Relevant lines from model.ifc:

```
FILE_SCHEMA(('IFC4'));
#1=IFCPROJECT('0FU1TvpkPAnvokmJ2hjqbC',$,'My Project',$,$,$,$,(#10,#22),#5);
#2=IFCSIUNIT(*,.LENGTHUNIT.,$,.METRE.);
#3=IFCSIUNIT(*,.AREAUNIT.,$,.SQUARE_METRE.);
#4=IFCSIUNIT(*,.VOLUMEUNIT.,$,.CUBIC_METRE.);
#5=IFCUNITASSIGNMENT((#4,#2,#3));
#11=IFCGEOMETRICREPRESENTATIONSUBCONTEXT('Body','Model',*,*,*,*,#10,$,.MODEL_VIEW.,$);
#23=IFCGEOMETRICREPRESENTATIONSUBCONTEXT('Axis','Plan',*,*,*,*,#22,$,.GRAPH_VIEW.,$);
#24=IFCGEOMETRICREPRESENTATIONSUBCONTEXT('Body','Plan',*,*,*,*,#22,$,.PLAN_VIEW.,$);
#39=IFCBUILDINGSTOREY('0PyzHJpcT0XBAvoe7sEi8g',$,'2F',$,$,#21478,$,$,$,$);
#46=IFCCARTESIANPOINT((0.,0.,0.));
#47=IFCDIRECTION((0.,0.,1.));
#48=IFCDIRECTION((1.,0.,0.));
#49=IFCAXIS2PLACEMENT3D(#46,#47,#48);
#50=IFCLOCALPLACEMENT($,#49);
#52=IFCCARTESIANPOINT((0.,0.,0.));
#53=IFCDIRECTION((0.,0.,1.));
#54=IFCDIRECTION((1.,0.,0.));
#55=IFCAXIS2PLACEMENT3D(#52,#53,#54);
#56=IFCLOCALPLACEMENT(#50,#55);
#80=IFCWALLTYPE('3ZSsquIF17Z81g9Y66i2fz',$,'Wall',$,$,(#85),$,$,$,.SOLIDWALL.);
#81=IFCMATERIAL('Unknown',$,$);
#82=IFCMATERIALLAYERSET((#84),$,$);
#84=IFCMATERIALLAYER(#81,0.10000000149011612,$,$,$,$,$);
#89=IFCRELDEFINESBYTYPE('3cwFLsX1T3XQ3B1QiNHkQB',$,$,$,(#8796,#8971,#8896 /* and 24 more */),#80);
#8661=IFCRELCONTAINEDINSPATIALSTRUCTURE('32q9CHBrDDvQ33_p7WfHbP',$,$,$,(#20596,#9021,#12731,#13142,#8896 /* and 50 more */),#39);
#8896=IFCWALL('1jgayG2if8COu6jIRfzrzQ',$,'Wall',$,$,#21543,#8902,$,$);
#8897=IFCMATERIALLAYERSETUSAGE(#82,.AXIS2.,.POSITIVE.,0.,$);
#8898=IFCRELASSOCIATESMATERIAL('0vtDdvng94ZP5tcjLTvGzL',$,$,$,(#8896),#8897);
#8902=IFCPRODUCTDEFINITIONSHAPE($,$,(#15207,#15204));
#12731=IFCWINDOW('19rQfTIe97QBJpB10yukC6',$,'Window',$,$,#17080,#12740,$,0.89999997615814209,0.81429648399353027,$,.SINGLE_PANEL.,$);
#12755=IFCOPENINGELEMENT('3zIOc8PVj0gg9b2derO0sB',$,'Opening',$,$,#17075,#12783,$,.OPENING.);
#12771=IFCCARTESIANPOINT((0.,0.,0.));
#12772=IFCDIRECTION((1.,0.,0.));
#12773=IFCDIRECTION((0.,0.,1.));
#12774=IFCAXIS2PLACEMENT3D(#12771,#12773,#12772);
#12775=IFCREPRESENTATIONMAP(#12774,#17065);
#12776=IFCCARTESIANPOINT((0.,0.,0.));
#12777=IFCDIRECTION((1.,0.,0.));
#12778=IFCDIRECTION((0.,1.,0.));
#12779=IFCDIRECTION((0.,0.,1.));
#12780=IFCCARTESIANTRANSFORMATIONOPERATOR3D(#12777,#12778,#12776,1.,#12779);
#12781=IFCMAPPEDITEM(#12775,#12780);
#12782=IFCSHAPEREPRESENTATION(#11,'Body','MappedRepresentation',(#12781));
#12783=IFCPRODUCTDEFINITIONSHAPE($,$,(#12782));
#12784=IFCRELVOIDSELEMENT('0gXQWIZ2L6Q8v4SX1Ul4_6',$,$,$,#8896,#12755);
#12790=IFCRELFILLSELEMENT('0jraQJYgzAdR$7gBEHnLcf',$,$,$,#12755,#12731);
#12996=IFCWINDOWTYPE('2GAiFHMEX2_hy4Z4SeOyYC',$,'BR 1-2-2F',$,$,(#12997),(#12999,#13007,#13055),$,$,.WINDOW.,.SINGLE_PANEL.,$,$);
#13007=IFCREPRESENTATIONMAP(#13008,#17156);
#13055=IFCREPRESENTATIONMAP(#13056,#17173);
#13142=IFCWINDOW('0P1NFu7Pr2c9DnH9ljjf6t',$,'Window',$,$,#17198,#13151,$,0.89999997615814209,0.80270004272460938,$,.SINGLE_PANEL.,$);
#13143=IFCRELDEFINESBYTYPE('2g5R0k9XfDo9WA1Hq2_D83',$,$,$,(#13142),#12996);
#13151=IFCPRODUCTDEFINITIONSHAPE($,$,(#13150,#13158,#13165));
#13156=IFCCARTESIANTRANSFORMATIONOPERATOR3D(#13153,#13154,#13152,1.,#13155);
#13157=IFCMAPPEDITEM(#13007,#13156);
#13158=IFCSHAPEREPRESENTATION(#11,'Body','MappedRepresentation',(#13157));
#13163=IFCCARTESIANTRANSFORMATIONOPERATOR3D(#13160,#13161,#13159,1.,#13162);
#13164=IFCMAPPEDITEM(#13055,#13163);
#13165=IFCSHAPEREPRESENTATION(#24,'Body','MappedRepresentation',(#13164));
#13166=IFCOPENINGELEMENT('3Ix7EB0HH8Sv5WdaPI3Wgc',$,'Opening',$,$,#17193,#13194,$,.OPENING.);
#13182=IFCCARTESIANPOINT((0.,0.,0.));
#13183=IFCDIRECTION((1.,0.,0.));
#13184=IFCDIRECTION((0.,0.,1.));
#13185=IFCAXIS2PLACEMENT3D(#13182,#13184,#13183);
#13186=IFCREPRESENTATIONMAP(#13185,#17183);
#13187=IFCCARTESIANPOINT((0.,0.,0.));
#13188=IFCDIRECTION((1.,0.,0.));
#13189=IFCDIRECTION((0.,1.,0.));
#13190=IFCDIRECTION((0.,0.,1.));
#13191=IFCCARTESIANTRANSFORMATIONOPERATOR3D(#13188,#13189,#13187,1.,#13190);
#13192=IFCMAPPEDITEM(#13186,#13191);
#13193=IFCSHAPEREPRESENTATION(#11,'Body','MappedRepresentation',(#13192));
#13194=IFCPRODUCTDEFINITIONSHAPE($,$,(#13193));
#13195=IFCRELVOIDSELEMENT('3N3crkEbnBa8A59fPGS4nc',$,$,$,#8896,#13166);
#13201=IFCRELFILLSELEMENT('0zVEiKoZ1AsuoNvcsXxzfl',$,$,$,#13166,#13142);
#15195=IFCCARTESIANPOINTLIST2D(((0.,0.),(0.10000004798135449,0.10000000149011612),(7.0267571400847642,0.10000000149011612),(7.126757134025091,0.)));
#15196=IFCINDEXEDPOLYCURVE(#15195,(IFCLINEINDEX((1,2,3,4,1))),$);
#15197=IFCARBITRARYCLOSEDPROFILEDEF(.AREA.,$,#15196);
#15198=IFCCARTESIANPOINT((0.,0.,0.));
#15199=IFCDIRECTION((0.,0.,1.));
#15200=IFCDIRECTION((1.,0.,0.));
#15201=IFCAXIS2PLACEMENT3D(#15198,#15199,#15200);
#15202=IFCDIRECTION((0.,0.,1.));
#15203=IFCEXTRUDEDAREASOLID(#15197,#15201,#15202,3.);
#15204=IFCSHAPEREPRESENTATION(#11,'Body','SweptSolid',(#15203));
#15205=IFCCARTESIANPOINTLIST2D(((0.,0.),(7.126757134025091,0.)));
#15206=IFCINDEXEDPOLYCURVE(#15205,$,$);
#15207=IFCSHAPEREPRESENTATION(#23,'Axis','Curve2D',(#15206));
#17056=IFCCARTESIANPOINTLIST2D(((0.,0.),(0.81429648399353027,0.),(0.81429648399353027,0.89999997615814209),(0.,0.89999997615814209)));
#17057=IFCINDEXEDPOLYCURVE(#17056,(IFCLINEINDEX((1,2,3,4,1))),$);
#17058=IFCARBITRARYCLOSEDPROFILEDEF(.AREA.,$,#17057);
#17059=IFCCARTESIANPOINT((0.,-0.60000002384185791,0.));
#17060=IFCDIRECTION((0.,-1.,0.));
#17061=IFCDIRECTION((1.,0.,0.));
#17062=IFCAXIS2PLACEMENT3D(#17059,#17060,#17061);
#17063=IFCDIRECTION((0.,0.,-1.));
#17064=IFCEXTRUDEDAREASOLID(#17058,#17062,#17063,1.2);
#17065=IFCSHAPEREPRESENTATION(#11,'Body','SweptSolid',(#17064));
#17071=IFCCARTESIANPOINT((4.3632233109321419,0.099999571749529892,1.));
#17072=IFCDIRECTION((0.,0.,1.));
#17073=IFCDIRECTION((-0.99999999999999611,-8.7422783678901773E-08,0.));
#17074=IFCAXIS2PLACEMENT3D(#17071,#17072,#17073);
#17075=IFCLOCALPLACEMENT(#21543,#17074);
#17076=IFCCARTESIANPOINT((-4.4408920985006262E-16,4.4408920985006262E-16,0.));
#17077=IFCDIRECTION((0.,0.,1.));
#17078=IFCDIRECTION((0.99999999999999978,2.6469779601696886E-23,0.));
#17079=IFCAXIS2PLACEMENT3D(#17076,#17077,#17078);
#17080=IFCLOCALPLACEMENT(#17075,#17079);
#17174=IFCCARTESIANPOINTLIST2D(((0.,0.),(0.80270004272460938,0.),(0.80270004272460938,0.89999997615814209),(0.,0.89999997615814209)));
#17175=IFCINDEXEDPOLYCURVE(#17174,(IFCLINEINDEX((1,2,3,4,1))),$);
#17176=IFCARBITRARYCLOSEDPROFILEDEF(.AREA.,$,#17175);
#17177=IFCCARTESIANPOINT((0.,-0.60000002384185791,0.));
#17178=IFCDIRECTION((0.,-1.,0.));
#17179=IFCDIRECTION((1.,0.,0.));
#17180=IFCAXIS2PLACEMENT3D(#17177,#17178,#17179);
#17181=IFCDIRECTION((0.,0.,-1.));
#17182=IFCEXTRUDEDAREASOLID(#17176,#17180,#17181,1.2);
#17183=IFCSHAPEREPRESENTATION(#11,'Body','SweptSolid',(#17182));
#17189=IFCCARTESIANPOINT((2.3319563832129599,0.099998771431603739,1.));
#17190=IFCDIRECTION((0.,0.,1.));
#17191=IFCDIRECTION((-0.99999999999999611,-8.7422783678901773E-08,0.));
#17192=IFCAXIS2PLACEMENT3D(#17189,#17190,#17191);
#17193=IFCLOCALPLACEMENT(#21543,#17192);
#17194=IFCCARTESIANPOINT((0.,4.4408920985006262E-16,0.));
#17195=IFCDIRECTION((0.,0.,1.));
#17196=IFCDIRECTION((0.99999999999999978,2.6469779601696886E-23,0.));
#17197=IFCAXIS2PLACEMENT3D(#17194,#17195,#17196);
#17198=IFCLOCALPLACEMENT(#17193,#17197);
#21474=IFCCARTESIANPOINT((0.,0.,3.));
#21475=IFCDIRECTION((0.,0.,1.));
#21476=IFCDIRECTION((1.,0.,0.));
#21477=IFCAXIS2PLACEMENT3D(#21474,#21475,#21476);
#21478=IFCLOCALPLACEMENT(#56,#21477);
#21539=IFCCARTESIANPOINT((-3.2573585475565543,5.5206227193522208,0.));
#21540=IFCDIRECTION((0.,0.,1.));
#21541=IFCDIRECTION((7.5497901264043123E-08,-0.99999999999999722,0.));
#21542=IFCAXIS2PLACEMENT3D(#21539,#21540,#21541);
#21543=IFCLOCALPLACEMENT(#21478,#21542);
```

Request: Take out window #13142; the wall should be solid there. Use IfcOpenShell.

```python
import ifcopenshell
import ifcopenshell.api.feature
import ifcopenshell.api.root
import ifcopenshell.geom
import ifcopenshell.util.shape

model = ifcopenshell.open("model.ifc")
settings = ifcopenshell.geom.settings()


def volume(element):
    """Net volume in cubic metres, openings subtracted."""
    shape = ifcopenshell.geom.create_shape(settings, element)
    return ifcopenshell.util.shape.get_volume(shape.geometry)


window = model.by_guid("0P1NFu7Pr2c9DnH9ljjf6t")
opening = window.FillsVoids[0].RelatingOpeningElement
wall = opening.VoidsElements[0].RelatingBuildingElement
before = volume(wall)

ifcopenshell.api.root.remove_product(model, product=window)
ifcopenshell.api.feature.remove_feature(model, feature=opening)

after = volume(wall)

print(f"wall volume {before:.3f} -> {after:.3f} m3")

model.write("model_updated.ifc")
```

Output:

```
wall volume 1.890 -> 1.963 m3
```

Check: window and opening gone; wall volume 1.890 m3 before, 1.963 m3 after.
